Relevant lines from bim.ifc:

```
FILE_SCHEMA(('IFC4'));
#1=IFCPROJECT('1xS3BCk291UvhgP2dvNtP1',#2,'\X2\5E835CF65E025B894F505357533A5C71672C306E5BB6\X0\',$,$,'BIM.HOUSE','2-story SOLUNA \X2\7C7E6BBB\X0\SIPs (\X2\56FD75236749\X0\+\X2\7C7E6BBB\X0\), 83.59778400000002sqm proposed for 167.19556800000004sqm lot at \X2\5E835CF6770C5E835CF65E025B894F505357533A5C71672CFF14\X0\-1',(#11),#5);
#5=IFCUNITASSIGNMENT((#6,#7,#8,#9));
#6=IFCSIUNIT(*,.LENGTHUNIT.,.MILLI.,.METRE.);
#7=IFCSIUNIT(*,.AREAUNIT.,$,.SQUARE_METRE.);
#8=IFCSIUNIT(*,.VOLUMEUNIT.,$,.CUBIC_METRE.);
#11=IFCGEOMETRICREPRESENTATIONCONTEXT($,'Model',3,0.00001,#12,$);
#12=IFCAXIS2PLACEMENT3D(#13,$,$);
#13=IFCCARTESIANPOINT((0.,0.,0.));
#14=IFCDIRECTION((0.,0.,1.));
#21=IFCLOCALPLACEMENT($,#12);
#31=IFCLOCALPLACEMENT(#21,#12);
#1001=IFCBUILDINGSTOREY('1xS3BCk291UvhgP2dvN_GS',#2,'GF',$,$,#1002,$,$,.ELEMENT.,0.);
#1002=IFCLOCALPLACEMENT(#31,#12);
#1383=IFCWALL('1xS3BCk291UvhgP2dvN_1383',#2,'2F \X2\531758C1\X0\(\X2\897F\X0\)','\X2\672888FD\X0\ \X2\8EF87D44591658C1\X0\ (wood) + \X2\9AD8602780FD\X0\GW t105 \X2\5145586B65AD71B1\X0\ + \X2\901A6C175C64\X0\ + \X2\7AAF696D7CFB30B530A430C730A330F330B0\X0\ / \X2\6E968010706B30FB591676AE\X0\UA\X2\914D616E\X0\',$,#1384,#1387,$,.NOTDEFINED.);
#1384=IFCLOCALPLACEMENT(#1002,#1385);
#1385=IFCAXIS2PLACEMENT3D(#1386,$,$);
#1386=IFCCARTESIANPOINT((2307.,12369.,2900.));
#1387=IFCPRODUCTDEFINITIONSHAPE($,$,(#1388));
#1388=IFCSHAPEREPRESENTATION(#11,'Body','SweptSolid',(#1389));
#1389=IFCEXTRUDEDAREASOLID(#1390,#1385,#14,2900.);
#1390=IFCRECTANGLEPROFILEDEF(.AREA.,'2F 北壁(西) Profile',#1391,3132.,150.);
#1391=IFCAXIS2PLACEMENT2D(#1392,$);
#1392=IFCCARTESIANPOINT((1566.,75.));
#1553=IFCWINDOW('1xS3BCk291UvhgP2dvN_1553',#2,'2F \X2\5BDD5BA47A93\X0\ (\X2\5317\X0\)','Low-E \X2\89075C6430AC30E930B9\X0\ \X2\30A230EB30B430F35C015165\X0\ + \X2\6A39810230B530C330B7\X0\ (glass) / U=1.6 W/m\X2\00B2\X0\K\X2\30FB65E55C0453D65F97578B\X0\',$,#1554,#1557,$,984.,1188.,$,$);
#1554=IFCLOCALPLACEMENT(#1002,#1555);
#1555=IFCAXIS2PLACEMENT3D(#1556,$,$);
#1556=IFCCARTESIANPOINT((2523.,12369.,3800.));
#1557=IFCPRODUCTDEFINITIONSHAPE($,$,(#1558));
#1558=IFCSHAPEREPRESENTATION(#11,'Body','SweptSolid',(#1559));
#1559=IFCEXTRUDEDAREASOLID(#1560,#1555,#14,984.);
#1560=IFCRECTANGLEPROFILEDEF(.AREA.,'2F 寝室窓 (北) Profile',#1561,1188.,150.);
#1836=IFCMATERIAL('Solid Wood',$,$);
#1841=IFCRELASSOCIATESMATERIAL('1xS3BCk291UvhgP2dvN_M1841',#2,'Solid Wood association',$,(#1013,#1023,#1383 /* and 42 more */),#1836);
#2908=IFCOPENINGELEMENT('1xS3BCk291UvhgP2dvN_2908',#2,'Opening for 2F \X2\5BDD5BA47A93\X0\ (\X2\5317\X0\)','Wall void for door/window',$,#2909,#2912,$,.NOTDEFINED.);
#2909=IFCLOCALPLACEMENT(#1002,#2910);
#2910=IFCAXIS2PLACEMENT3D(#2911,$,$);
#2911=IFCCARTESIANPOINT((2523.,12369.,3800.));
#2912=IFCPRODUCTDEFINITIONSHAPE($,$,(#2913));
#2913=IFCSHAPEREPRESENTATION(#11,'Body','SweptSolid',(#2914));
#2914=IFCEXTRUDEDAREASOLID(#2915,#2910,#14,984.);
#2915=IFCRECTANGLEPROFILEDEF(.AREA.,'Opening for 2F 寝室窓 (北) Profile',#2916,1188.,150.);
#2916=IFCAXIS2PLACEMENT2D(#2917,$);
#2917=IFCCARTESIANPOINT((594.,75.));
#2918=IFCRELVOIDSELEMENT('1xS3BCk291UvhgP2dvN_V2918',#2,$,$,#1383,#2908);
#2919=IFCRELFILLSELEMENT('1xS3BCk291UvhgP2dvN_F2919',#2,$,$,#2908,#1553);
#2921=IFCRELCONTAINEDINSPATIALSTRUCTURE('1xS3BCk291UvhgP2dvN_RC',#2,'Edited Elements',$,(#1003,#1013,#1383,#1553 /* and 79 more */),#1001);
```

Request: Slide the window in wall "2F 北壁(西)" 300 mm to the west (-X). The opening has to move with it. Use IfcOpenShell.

```python
import ifcopenshell
import ifcopenshell.api.geometry
import ifcopenshell.util.placement

model = ifcopenshell.open("bim.ifc")

window = model.by_guid("1xS3BCk291UvhgP2dvN_1553")
opening = window.FillsVoids[0].RelatingOpeningElement
wall = opening.VoidsElements[0].RelatingBuildingElement

wall_matrix = ifcopenshell.util.placement.get_local_placement(wall.ObjectPlacement)
shift = wall_matrix[:3, 0] * -300.0
before = ifcopenshell.util.placement.get_local_placement(window.ObjectPlacement)[:3, 3].copy()

# The window is not placed relative to its opening, so move both.
for product in (opening, window):
    matrix = ifcopenshell.util.placement.get_local_placement(product.ObjectPlacement)
    matrix[:3, 3] += shift
    ifcopenshell.api.geometry.edit_object_placement(model, product=product, matrix=matrix, is_si=False)

after = ifcopenshell.util.placement.get_local_placement(window.ObjectPlacement)[:3, 3]
print("window moved by", (after - before).round(3) + 0.0)

model.write("bim_edited.ifc")
```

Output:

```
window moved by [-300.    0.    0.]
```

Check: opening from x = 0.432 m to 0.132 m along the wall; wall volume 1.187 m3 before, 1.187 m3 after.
